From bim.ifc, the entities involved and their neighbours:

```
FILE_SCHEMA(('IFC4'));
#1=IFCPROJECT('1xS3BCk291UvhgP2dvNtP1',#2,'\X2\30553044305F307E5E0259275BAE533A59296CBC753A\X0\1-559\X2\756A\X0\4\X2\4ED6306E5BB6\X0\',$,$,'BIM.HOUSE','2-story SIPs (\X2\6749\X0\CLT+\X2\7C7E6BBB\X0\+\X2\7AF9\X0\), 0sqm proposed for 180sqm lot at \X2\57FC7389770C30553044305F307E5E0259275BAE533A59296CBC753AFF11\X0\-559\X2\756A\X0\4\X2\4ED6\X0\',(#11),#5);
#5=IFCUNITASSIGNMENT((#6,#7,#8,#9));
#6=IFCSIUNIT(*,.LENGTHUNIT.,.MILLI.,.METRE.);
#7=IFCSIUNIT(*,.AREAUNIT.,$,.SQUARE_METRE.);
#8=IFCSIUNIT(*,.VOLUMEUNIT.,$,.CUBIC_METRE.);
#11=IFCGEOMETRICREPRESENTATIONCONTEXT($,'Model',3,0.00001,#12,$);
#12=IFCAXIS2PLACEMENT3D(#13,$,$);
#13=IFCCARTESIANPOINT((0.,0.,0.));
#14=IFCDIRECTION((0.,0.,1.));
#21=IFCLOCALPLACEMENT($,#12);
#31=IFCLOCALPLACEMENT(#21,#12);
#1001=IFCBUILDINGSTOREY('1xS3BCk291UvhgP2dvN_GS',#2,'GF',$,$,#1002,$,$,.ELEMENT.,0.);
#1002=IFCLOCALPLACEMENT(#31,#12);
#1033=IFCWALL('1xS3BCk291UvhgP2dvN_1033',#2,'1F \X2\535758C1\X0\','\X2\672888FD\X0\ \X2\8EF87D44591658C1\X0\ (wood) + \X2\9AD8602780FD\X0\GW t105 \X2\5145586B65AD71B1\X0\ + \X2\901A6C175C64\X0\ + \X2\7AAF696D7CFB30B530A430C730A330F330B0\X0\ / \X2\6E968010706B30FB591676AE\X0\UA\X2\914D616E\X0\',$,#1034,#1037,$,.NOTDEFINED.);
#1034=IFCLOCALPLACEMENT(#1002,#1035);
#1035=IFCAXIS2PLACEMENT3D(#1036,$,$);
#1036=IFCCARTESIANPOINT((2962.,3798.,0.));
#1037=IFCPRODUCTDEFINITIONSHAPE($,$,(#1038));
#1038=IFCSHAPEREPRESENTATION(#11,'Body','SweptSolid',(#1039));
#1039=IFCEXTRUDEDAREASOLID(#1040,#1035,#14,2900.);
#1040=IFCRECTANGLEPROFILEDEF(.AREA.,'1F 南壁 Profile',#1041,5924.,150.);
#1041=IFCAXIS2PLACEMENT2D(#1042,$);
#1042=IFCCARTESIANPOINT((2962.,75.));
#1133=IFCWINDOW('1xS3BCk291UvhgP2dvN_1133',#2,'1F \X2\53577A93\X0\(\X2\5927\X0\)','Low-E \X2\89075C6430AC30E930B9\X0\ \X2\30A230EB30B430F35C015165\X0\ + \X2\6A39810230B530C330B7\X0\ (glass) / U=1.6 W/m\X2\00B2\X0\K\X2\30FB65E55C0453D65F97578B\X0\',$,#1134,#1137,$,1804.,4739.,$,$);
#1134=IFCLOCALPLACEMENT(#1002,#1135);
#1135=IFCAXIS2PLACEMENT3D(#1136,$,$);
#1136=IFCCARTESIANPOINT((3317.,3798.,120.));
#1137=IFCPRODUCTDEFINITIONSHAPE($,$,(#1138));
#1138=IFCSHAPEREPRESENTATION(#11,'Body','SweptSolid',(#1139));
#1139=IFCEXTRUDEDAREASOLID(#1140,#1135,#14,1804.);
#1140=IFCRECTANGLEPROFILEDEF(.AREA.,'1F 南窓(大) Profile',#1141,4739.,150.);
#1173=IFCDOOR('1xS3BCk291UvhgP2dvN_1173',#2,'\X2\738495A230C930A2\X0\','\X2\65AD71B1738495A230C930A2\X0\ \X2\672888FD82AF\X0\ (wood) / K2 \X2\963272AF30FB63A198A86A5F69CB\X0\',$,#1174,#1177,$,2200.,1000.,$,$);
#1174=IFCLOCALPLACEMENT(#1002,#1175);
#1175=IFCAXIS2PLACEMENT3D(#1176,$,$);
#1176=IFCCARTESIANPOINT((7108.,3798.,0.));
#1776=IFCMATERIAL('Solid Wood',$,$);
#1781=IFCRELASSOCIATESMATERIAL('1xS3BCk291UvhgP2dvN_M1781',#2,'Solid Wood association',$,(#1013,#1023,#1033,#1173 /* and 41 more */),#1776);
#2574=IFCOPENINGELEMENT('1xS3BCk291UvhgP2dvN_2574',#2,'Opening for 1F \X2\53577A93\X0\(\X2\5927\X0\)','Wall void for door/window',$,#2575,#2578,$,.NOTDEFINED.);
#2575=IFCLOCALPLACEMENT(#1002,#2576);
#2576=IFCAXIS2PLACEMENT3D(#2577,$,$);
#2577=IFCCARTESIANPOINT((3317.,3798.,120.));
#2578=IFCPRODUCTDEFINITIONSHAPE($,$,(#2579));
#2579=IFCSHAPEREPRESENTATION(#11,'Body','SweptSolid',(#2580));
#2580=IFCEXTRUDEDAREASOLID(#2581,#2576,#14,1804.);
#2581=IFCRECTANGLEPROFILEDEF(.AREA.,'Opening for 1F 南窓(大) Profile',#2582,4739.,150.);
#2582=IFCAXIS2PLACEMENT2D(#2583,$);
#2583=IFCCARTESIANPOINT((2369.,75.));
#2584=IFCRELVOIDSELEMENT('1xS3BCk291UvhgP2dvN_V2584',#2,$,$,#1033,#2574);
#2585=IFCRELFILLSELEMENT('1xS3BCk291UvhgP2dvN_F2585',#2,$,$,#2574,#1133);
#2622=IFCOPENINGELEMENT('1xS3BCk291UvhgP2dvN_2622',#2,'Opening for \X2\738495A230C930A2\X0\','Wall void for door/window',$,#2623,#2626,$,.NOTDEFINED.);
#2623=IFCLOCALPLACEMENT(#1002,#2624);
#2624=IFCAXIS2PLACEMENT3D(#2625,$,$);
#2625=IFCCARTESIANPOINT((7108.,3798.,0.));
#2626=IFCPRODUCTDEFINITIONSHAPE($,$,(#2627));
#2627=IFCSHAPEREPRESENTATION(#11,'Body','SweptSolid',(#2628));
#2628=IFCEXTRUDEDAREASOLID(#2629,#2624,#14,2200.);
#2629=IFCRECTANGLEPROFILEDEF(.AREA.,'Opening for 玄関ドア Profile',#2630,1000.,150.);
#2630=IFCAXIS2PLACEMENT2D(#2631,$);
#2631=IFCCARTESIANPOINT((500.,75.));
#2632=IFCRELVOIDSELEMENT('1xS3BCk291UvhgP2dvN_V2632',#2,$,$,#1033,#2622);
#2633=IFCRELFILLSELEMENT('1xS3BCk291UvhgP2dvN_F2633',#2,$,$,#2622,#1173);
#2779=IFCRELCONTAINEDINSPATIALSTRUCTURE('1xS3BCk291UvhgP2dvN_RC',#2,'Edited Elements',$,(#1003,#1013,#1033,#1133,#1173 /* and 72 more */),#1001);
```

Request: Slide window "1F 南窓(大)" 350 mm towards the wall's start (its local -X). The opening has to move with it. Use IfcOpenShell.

```python
import ifcopenshell
import ifcopenshell.api.geometry
import ifcopenshell.util.placement
import ifcopenshell.util.unit

model = ifcopenshell.open("bim.ifc")
unit_scale = ifcopenshell.util.unit.calculate_unit_scale(model)

window = model.by_guid("1xS3BCk291UvhgP2dvN_1133")
opening = window.FillsVoids[0].RelatingOpeningElement
wall = opening.VoidsElements[0].RelatingBuildingElement

wall_matrix = ifcopenshell.util.placement.get_local_placement(wall.ObjectPlacement)
shift = wall_matrix[:3, 0] * -0.35 / unit_scale
before = ifcopenshell.util.placement.get_local_placement(window.ObjectPlacement)[:3, 3].copy()

# The window is not placed relative to its opening, so move both.
for product in (opening, window):
    matrix = ifcopenshell.util.placement.get_local_placement(product.ObjectPlacement)
    matrix[:3, 3] += shift
    ifcopenshell.api.geometry.edit_object_placement(model, product=product, matrix=matrix, is_si=False)

after = ifcopenshell.util.placement.get_local_placement(window.ObjectPlacement)[:3, 3]
print("window moved by", (after - before).round(3) + 0.0)

model.write("bim_edited.ifc")
```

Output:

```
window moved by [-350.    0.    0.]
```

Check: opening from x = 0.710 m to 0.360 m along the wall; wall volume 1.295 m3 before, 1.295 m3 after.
